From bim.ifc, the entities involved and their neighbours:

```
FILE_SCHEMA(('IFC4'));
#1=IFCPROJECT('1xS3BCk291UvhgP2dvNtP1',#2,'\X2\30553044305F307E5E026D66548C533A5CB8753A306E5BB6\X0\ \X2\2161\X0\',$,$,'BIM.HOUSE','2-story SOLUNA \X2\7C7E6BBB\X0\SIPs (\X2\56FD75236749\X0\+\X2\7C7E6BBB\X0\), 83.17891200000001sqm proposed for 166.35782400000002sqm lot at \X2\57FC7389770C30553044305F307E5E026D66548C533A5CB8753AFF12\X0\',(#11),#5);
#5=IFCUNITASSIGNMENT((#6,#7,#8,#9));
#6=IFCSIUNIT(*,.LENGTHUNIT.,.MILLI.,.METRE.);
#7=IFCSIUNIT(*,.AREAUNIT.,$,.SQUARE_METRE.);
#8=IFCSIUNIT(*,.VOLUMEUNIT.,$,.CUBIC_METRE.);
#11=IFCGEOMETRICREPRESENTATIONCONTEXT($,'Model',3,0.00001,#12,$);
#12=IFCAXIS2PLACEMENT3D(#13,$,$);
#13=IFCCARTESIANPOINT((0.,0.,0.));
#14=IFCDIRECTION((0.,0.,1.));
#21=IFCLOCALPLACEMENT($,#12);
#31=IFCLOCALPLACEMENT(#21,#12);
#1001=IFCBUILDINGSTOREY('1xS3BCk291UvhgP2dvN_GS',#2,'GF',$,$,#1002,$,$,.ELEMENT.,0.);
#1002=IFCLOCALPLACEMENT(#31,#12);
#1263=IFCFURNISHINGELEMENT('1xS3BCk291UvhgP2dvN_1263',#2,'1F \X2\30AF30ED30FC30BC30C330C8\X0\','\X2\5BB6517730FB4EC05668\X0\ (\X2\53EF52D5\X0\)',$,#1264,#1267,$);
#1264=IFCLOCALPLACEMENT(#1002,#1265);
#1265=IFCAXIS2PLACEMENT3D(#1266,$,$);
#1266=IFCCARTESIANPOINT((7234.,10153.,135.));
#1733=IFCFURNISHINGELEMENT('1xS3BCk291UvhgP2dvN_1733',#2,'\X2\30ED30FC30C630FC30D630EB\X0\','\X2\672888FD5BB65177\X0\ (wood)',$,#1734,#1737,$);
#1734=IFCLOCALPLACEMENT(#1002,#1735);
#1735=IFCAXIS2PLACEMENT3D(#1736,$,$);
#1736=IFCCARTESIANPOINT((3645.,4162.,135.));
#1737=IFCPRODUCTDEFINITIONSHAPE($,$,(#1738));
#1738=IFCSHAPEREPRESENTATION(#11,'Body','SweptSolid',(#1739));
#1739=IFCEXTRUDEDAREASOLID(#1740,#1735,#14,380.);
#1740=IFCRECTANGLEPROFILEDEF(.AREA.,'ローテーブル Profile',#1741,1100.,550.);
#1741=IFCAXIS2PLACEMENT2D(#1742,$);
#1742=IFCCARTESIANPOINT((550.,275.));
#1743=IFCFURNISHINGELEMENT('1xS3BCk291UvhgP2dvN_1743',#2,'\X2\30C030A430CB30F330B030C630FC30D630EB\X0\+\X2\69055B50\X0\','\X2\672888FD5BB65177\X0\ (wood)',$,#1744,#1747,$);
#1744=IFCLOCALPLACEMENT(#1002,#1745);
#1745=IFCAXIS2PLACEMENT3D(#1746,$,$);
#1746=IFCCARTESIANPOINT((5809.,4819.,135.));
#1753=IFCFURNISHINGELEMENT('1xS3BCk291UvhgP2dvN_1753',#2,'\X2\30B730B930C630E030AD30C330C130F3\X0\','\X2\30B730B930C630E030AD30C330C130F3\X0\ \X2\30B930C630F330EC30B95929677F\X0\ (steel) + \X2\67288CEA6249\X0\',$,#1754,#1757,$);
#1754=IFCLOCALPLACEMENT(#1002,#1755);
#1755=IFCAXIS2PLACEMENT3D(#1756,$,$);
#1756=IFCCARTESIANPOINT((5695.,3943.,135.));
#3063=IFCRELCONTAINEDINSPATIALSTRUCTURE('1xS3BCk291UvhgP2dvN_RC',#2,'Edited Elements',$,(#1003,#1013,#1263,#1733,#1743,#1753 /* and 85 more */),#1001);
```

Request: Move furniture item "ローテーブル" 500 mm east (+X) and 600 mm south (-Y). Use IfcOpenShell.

```python
import ifcopenshell
import ifcopenshell.api.geometry
import ifcopenshell.util.placement
import ifcopenshell.util.unit

model = ifcopenshell.open("bim.ifc")
unit_scale = ifcopenshell.util.unit.calculate_unit_scale(model)

item = model.by_guid("1xS3BCk291UvhgP2dvN_1733")
matrix = ifcopenshell.util.placement.get_local_placement(item.ObjectPlacement)
matrix[0, 3] += 0.5 / unit_scale
matrix[1, 3] -= 0.6 / unit_scale
ifcopenshell.api.geometry.edit_object_placement(model, product=item, matrix=matrix, is_si=False)

print(ifcopenshell.util.placement.get_local_placement(item.ObjectPlacement).round(3) + 0.0)

model.write("bim_v2.ifc")
```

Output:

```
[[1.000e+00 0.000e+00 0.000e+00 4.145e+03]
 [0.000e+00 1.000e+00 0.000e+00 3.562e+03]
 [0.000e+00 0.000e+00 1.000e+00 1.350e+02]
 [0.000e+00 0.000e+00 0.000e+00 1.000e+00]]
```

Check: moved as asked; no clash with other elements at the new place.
